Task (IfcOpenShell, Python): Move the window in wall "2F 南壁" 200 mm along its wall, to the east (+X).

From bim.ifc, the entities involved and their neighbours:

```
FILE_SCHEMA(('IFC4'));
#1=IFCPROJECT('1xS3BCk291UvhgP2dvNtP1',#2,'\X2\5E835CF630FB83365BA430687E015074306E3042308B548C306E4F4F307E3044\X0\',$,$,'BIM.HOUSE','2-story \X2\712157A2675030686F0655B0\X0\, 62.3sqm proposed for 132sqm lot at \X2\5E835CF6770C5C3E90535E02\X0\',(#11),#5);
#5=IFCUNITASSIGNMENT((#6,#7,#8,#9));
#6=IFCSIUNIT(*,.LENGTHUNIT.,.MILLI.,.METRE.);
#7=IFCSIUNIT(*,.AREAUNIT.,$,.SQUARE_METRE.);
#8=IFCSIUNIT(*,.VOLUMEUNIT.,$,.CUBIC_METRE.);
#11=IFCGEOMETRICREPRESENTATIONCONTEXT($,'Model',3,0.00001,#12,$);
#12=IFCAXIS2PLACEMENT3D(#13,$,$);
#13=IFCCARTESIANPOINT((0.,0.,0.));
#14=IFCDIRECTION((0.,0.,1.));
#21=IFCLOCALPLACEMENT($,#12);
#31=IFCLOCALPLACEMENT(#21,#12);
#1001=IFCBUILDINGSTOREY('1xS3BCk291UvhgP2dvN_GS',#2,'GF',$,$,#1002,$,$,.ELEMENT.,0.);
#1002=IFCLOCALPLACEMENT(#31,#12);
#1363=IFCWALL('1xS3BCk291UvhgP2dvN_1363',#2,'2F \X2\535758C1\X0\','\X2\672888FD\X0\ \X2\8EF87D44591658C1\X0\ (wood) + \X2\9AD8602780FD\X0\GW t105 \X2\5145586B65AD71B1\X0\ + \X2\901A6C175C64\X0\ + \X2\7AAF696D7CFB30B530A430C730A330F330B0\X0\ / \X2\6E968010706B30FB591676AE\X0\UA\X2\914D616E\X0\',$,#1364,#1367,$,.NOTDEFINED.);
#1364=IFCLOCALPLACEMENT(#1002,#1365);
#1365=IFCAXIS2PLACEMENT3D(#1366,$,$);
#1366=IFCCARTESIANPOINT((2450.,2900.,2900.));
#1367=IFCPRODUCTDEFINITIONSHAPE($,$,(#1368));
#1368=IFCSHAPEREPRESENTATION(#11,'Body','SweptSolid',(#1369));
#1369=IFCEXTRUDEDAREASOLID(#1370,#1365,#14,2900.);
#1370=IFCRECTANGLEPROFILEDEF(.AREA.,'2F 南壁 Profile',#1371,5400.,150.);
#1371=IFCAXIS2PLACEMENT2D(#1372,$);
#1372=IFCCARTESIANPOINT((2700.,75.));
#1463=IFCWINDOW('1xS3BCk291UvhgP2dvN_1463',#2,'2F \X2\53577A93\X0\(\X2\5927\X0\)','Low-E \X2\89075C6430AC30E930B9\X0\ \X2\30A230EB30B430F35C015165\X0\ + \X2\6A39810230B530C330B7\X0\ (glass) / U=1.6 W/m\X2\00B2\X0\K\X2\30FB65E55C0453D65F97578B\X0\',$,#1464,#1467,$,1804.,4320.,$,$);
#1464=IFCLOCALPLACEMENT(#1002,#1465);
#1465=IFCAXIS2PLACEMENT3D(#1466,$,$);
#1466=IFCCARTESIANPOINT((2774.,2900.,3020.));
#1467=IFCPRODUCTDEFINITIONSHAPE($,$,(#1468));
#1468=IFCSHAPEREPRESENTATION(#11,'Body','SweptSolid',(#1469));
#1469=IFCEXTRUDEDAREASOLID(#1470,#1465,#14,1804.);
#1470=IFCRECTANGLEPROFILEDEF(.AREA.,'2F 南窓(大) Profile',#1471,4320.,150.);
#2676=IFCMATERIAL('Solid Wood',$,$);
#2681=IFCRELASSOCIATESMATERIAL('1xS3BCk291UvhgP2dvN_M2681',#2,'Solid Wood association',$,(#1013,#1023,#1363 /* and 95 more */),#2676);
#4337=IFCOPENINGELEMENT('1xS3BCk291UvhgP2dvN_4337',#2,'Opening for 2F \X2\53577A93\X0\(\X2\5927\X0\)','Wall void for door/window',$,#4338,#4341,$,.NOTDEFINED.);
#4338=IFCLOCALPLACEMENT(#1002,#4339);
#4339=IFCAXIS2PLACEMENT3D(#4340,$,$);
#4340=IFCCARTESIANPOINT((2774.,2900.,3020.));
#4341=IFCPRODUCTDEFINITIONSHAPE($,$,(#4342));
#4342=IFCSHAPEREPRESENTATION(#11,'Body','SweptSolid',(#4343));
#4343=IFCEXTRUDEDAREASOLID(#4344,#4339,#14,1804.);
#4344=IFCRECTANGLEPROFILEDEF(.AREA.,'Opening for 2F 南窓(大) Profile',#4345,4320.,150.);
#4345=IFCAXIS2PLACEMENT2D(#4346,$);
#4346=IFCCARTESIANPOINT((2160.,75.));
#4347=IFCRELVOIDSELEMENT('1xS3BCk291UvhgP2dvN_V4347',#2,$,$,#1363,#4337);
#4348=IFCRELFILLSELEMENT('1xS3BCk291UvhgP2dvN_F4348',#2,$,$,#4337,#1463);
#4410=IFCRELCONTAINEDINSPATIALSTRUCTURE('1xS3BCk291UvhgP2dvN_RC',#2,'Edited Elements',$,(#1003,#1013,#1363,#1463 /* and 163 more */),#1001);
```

```python
import ifcopenshell
import ifcopenshell.api.geometry
import ifcopenshell.util.placement
import ifcopenshell.util.unit

model = ifcopenshell.open("bim.ifc")
unit_scale = ifcopenshell.util.unit.calculate_unit_scale(model)

window = model.by_guid("1xS3BCk291UvhgP2dvN_1463")
opening = window.FillsVoids[0].RelatingOpeningElement
wall = opening.VoidsElements[0].RelatingBuildingElement

wall_matrix = ifcopenshell.util.placement.get_local_placement(wall.ObjectPlacement)
shift = wall_matrix[:3, 0] * 0.2 / unit_scale
before = ifcopenshell.util.placement.get_local_placement(window.ObjectPlacement)[:3, 3].copy()

# The window is not placed relative to its opening, so move both.
for product in (opening, window):
    matrix = ifcopenshell.util.placement.get_local_placement(product.ObjectPlacement)
    matrix[:3, 3] += shift
    ifcopenshell.api.geometry.edit_object_placement(model, product=product, matrix=matrix, is_si=False)

after = ifcopenshell.util.placement.get_local_placement(window.ObjectPlacement)[:3, 3]
print("window moved by", (after - before).round(3) + 0.0)

model.write("bim_rev.ifc")
```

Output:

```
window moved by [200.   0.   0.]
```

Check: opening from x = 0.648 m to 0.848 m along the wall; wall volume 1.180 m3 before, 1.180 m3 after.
